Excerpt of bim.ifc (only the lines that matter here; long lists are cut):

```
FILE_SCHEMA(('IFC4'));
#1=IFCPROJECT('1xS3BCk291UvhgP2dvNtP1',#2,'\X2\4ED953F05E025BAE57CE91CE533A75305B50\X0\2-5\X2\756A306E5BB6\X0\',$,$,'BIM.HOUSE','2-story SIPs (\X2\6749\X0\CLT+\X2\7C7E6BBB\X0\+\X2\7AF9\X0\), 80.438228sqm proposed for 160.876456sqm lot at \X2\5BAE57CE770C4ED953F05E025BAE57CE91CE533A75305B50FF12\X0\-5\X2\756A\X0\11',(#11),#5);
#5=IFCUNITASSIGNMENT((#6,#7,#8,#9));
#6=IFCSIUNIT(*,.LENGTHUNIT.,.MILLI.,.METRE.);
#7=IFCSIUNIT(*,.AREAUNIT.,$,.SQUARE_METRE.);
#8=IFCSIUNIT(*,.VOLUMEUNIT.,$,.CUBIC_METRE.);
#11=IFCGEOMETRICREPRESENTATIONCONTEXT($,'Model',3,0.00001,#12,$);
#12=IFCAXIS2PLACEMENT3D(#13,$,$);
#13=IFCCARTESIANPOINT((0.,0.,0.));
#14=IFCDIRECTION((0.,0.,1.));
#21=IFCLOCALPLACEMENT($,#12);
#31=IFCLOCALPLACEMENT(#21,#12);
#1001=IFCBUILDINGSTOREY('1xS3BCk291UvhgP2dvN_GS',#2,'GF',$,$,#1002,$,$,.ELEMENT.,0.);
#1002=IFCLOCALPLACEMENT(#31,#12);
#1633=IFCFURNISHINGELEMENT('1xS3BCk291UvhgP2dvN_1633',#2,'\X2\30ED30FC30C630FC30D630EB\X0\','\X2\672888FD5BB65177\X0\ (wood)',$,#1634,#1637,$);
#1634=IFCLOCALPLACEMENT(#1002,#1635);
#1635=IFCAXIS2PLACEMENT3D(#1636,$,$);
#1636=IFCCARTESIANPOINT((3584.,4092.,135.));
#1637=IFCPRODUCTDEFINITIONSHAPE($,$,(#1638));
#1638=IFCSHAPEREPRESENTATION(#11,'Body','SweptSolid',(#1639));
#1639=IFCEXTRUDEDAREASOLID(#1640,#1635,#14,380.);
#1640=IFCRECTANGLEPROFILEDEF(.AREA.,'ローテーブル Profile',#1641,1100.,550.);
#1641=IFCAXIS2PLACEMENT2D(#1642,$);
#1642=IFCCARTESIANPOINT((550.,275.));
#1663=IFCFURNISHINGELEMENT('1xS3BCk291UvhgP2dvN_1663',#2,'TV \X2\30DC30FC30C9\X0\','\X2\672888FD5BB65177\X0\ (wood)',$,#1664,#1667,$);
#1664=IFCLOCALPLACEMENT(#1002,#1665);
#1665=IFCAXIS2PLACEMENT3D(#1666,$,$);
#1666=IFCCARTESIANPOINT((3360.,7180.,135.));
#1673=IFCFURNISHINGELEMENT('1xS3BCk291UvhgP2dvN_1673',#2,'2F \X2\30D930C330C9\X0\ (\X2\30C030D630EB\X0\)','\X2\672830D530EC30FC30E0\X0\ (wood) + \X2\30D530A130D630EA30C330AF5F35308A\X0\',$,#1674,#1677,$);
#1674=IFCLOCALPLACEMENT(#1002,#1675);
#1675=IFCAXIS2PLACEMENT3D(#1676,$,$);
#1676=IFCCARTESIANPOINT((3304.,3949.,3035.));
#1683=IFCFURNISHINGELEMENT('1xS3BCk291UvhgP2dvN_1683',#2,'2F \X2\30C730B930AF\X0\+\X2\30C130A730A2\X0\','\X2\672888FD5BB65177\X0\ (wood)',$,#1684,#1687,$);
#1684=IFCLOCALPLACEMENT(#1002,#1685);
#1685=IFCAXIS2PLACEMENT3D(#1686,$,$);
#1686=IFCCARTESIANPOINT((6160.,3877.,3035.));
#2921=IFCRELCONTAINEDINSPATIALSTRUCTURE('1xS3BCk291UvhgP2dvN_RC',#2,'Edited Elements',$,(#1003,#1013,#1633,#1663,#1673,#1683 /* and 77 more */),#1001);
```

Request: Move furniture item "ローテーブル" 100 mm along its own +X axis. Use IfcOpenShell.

```python
import ifcopenshell
import ifcopenshell.api.geometry
import ifcopenshell.util.placement
import ifcopenshell.util.unit

model = ifcopenshell.open("bim.ifc")
unit_scale = ifcopenshell.util.unit.calculate_unit_scale(model)

item = model.by_guid("1xS3BCk291UvhgP2dvN_1633")
matrix = ifcopenshell.util.placement.get_local_placement(item.ObjectPlacement)
matrix[:3, 3] += matrix[:3, 0] * 0.1 / unit_scale
ifcopenshell.api.geometry.edit_object_placement(model, product=item, matrix=matrix, is_si=False)

print(ifcopenshell.util.placement.get_local_placement(item.ObjectPlacement).round(3) + 0.0)

model.write("bim_updated.ifc")
```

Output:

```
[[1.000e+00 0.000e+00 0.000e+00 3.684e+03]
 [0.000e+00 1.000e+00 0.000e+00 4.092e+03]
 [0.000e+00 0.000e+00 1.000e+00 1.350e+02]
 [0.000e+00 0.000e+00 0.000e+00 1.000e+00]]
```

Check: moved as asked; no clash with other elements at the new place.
